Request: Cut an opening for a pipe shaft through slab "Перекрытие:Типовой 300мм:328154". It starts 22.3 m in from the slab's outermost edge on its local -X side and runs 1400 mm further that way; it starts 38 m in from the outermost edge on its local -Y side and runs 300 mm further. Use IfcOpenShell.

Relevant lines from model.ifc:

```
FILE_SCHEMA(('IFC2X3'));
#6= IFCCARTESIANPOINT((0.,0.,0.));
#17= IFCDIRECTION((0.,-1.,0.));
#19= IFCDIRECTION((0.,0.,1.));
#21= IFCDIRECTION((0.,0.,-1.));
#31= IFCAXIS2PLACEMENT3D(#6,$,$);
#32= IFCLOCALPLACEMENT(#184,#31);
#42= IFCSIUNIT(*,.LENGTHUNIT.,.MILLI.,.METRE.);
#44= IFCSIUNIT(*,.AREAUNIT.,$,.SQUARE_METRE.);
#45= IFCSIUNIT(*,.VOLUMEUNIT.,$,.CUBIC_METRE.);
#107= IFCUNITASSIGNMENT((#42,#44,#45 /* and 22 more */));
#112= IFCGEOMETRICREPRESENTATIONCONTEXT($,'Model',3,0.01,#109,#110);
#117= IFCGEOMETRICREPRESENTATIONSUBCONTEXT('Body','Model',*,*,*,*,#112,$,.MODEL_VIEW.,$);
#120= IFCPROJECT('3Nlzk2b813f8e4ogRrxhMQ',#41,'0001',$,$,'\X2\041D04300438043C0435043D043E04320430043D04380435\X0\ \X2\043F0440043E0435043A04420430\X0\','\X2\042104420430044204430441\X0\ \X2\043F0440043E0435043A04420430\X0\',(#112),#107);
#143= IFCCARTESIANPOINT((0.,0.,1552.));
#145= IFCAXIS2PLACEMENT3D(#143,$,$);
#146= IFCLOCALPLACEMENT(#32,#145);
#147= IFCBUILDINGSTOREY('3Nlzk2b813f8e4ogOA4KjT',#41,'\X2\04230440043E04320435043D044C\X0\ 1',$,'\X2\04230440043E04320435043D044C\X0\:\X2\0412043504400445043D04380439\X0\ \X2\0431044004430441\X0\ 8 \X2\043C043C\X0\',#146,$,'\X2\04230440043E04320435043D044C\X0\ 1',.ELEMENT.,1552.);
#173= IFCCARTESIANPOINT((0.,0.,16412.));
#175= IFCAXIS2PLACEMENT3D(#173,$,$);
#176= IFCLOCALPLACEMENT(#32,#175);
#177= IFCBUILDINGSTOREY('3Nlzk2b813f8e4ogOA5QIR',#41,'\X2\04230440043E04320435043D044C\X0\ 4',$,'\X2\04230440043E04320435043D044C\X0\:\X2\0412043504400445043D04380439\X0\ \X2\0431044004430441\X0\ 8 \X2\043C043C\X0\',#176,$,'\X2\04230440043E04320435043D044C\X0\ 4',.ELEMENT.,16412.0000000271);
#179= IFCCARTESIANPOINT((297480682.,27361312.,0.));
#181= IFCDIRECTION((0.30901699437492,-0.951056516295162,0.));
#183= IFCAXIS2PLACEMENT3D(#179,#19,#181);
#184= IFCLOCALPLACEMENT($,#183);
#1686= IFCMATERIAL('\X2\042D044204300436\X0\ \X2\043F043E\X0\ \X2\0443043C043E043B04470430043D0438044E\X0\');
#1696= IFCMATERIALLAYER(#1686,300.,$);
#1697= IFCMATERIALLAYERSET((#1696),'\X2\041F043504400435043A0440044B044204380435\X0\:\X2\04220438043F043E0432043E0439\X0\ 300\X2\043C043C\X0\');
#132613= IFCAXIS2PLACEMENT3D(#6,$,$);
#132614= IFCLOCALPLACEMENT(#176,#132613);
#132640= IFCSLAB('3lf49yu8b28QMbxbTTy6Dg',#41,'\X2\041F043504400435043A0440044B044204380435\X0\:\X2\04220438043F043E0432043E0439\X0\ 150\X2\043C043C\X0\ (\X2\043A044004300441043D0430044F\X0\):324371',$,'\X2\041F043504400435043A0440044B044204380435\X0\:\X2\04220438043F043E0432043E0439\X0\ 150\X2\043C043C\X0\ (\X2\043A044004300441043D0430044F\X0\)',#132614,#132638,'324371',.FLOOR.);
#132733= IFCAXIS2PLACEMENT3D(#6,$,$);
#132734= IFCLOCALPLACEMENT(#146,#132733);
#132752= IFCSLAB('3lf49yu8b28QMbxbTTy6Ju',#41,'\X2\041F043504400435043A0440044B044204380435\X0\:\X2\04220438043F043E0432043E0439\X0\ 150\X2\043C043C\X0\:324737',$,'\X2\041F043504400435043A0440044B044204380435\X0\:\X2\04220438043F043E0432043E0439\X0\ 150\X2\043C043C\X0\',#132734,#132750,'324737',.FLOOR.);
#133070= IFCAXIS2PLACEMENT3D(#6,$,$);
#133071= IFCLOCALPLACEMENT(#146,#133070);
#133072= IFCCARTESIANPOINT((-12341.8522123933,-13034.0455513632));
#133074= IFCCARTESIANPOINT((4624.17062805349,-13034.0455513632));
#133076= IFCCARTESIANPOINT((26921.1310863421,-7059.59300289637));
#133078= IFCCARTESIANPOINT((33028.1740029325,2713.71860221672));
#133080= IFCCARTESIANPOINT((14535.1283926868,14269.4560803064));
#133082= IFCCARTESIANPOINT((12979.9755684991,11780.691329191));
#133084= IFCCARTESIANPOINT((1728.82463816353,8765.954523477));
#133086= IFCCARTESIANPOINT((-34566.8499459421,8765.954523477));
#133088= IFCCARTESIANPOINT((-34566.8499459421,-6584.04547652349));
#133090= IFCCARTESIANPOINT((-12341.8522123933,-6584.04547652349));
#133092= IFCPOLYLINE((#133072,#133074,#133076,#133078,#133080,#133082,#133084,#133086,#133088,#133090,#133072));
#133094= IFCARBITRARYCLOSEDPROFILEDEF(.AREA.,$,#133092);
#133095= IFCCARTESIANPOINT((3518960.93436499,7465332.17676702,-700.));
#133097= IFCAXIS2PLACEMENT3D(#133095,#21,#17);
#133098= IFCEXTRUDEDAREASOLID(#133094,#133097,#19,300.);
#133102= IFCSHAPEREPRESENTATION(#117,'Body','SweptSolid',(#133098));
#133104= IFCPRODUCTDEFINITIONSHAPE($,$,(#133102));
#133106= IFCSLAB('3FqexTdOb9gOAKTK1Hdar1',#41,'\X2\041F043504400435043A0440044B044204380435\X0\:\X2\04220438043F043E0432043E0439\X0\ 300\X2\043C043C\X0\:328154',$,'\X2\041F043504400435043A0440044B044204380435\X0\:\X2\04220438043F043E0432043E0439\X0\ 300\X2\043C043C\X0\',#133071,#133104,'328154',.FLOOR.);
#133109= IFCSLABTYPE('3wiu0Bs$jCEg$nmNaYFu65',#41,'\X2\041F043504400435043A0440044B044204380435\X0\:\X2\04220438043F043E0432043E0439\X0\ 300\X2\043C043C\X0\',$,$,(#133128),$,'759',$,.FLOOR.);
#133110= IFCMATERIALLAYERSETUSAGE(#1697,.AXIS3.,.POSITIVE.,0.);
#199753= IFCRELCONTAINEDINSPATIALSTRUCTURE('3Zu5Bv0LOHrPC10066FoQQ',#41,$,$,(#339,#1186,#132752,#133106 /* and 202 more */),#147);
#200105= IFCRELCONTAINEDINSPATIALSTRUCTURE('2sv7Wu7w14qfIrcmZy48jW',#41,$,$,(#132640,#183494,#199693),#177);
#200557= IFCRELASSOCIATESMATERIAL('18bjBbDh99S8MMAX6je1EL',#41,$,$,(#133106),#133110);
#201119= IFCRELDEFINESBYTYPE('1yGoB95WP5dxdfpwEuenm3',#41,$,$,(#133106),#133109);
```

```python
import numpy as np
import ifcopenshell
import ifcopenshell.api.feature
import ifcopenshell.api.geometry
import ifcopenshell.api.root
import ifcopenshell.geom
import ifcopenshell.util.placement
import ifcopenshell.util.representation
import ifcopenshell.util.shape
import ifcopenshell.util.unit

model = ifcopenshell.open("model.ifc")
unit_scale = ifcopenshell.util.unit.calculate_unit_scale(model)
settings = ifcopenshell.geom.settings()


def volume(element):
    """Net volume in cubic metres, openings subtracted."""
    shape = ifcopenshell.geom.create_shape(settings, element)
    return ifcopenshell.util.shape.get_volume(shape.geometry)


slab = model.by_guid("3FqexTdOb9gOAKTK1Hdar1")
before = volume(slab)

# Extent in the slab's own axes, in metres. The edges named are its -X and -Y sides.
slab_shape = ifcopenshell.geom.create_shape(settings, slab)
vertices = ifcopenshell.util.shape.get_vertices(slab_shape.geometry)
x_min, y_min, bottom = vertices.min(axis=0)
top = vertices[:, 2].max()

opening = ifcopenshell.api.root.create_entity(model, ifc_class="IfcOpeningElement", name="Pipe shaft opening")
context = ifcopenshell.util.representation.get_context(model, "Model", "Body", "MODEL_VIEW")
width, depth = 1.4, 0.3
outline = [(0.0, 0.0), (width, 0.0), (width, depth), (0.0, depth), (0.0, 0.0)]
# Overshoot both faces by 50 mm so the cut is clean.
shape = ifcopenshell.api.geometry.add_slab_representation(
    model, context=context, depth=top - bottom + 0.1, polyline=outline
)
ifcopenshell.api.geometry.assign_representation(model, product=opening, representation=shape)

matrix = ifcopenshell.util.placement.get_local_placement(slab.ObjectPlacement)
matrix[:, 3] = matrix @ np.append(np.array([x_min + 22.3, y_min + 38, bottom - 0.05]) / unit_scale, 1.0)
ifcopenshell.api.geometry.edit_object_placement(model, product=opening, matrix=matrix, is_si=False)
ifcopenshell.api.feature.add_feature(model, feature=opening, element=slab)

after = volume(slab)

print(f"slab volume {before:.3f} -> {after:.3f} m3")

model.write("model_rev.ifc")
```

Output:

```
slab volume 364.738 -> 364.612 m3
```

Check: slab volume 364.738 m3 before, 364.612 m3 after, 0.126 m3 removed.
